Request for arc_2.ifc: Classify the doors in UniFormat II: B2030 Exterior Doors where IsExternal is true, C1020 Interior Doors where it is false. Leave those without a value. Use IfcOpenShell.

First a look at what the model holds.

```python
import ifcopenshell
import ifcopenshell.util.element

model = ifcopenshell.open("arc_2.ifc")
print(model.schema)
print("classifications:", [c.Name for c in model.by_type("IfcClassification")])
values = [ifcopenshell.util.element.get_pset(e, "Pset_DoorCommon", "IsExternal") for e in model.by_type("IfcDoor")]
for value in (True, False, None):
    print("IsExternal", value, values.count(value))
```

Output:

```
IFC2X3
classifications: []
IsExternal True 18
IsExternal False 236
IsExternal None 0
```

```python
import ifcopenshell
import ifcopenshell.api.classification
import ifcopenshell.util.element

model = ifcopenshell.open("arc_2.ifc")

# IFC2X3 requires Source and Edition and has no link from the project to the system.
system = model.create_entity("IfcClassification", Source="ASTM", Edition="E1557", Name="UniFormat II")

doors = model.by_type("IfcDoor")
external = {e: ifcopenshell.util.element.get_pset(e, "Pset_DoorCommon", "IsExternal") for e in doors}
for flag, code, name in ((True, "B2030", "Exterior Doors"), (False, "C1020", "Interior Doors")):
    products = [e for e in doors if external[e] is flag]
    ifcopenshell.api.classification.add_reference(
        model, products=products, classification=system, identification=code, name=name
    )
    print(code, len(products))

model.write("arc_2-out.ifc")
```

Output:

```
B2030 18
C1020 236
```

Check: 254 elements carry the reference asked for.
